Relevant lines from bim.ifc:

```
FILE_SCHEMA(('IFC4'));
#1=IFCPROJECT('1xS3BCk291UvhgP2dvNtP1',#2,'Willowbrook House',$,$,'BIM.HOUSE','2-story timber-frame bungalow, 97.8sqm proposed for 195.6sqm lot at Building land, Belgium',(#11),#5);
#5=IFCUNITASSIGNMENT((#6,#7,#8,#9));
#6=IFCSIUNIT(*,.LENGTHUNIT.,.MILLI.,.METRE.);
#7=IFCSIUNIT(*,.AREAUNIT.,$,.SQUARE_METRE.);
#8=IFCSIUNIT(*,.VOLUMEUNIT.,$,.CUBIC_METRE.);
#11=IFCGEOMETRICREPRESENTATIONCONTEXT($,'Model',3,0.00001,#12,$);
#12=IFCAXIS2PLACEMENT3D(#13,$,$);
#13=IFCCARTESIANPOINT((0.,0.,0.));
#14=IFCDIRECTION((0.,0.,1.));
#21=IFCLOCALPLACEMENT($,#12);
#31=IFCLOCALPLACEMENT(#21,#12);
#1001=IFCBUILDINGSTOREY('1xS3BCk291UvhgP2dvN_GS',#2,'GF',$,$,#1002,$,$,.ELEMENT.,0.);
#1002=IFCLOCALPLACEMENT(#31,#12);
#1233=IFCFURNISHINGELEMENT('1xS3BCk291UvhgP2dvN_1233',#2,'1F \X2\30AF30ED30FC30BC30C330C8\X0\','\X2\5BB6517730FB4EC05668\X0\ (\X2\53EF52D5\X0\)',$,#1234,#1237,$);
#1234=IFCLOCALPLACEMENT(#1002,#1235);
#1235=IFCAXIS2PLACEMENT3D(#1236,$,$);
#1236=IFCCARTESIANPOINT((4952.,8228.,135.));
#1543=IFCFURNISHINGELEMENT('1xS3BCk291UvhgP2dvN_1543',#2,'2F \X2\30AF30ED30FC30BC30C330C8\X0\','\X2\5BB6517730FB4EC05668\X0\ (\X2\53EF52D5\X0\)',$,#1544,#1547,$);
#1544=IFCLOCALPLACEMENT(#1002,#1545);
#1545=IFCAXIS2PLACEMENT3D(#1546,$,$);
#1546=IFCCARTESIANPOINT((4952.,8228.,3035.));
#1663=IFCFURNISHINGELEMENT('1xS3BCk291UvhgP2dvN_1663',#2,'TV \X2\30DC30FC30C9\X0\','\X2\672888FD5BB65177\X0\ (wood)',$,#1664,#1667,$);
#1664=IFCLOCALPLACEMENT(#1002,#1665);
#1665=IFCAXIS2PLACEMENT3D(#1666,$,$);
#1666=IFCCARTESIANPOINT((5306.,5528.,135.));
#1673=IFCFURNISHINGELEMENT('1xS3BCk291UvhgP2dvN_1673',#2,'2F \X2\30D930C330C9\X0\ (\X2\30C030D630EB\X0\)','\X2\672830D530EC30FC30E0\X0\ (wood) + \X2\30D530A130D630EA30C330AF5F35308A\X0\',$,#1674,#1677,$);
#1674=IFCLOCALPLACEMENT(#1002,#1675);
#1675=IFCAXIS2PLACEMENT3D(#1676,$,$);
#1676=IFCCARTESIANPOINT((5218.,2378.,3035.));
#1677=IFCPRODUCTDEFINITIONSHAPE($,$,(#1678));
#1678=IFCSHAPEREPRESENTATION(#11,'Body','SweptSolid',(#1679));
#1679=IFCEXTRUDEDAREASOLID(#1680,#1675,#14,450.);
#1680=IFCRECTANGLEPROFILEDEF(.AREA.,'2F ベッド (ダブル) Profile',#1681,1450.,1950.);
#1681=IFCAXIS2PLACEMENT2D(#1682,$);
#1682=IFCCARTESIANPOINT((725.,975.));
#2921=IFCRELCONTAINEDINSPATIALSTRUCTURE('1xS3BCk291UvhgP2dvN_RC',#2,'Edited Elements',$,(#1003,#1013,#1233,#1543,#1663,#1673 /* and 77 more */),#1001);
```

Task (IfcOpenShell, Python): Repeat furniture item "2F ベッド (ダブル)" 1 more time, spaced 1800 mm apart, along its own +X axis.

```python
import ifcopenshell
import ifcopenshell.api.geometry
import ifcopenshell.api.root
import ifcopenshell.util.element
import ifcopenshell.util.placement

model = ifcopenshell.open("bim.ifc")


def reuse_history(source, copy):
    """copy_class also copies each property set's owner history, people and application; keep the originals."""
    for rel in copy.IsDefinedBy:
        if rel.is_a("IfcRelDefinesByProperties") and (history := rel.RelatingPropertyDefinition.OwnerHistory):
            rel.RelatingPropertyDefinition.OwnerHistory = source.OwnerHistory
            ifcopenshell.util.element.remove_deep2(model, history)


source = model.by_guid("1xS3BCk291UvhgP2dvN_1673")
base = ifcopenshell.util.placement.get_local_placement(source.ObjectPlacement)
step = base[:3, 0] * 1800.0

for i in range(1, 2):
    copy = ifcopenshell.api.root.copy_class(model, product=source)
    copy.Representation = ifcopenshell.util.element.copy_deep(
        model, source.Representation, exclude=["IfcGeometricRepresentationContext", "IfcRepresentationMap"]
    )
    reuse_history(source, copy)
    matrix = base.copy()
    matrix[:3, 3] += i * step
    print("added at", matrix[:3, 3].round(3) + 0.0)
    ifcopenshell.api.geometry.edit_object_placement(model, product=copy, matrix=matrix, is_si=False)

model.write("bim_rev.ifc")
```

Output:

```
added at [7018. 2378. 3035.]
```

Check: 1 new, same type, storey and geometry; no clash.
